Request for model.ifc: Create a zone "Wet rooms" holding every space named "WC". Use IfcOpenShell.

First a look at what the model holds.

```python
import ifcopenshell

model = ifcopenshell.open("model.ifc")
print(model.schema)
seen = {}
for space in model.by_type("IfcSpace"):
    seen[space.LongName] = seen.get(space.LongName, 0) + 1
for name, count in sorted(seen.items(), key=str):
    print(count, "x", name)
print("zones:", [z.Name for z in model.by_type("IfcZone")][:20])
```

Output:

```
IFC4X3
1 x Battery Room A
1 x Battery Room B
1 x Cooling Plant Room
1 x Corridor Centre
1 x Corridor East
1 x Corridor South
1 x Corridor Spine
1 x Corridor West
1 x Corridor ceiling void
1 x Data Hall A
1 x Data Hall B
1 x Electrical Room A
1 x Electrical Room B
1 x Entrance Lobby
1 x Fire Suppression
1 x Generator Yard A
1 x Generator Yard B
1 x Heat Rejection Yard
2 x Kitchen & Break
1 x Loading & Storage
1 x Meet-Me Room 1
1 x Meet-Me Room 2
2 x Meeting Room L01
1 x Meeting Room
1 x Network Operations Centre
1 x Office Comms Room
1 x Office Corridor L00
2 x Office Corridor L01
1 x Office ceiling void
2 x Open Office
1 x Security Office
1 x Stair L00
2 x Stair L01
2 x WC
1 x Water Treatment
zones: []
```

```python
import ifcopenshell
import ifcopenshell.api.group
import ifcopenshell.api.root

model = ifcopenshell.open("model.ifc")

names = {"WC"}
spaces = [s for s in model.by_type("IfcSpace") if s.LongName in names]

zone = ifcopenshell.api.root.create_entity(model, ifc_class="IfcZone", name="Wet rooms")
ifcopenshell.api.group.assign_group(model, products=spaces, group=zone)
print(len(spaces), "spaces in", zone.Name)

model.write("model_rev.ifc")
```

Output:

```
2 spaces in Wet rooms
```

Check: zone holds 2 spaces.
